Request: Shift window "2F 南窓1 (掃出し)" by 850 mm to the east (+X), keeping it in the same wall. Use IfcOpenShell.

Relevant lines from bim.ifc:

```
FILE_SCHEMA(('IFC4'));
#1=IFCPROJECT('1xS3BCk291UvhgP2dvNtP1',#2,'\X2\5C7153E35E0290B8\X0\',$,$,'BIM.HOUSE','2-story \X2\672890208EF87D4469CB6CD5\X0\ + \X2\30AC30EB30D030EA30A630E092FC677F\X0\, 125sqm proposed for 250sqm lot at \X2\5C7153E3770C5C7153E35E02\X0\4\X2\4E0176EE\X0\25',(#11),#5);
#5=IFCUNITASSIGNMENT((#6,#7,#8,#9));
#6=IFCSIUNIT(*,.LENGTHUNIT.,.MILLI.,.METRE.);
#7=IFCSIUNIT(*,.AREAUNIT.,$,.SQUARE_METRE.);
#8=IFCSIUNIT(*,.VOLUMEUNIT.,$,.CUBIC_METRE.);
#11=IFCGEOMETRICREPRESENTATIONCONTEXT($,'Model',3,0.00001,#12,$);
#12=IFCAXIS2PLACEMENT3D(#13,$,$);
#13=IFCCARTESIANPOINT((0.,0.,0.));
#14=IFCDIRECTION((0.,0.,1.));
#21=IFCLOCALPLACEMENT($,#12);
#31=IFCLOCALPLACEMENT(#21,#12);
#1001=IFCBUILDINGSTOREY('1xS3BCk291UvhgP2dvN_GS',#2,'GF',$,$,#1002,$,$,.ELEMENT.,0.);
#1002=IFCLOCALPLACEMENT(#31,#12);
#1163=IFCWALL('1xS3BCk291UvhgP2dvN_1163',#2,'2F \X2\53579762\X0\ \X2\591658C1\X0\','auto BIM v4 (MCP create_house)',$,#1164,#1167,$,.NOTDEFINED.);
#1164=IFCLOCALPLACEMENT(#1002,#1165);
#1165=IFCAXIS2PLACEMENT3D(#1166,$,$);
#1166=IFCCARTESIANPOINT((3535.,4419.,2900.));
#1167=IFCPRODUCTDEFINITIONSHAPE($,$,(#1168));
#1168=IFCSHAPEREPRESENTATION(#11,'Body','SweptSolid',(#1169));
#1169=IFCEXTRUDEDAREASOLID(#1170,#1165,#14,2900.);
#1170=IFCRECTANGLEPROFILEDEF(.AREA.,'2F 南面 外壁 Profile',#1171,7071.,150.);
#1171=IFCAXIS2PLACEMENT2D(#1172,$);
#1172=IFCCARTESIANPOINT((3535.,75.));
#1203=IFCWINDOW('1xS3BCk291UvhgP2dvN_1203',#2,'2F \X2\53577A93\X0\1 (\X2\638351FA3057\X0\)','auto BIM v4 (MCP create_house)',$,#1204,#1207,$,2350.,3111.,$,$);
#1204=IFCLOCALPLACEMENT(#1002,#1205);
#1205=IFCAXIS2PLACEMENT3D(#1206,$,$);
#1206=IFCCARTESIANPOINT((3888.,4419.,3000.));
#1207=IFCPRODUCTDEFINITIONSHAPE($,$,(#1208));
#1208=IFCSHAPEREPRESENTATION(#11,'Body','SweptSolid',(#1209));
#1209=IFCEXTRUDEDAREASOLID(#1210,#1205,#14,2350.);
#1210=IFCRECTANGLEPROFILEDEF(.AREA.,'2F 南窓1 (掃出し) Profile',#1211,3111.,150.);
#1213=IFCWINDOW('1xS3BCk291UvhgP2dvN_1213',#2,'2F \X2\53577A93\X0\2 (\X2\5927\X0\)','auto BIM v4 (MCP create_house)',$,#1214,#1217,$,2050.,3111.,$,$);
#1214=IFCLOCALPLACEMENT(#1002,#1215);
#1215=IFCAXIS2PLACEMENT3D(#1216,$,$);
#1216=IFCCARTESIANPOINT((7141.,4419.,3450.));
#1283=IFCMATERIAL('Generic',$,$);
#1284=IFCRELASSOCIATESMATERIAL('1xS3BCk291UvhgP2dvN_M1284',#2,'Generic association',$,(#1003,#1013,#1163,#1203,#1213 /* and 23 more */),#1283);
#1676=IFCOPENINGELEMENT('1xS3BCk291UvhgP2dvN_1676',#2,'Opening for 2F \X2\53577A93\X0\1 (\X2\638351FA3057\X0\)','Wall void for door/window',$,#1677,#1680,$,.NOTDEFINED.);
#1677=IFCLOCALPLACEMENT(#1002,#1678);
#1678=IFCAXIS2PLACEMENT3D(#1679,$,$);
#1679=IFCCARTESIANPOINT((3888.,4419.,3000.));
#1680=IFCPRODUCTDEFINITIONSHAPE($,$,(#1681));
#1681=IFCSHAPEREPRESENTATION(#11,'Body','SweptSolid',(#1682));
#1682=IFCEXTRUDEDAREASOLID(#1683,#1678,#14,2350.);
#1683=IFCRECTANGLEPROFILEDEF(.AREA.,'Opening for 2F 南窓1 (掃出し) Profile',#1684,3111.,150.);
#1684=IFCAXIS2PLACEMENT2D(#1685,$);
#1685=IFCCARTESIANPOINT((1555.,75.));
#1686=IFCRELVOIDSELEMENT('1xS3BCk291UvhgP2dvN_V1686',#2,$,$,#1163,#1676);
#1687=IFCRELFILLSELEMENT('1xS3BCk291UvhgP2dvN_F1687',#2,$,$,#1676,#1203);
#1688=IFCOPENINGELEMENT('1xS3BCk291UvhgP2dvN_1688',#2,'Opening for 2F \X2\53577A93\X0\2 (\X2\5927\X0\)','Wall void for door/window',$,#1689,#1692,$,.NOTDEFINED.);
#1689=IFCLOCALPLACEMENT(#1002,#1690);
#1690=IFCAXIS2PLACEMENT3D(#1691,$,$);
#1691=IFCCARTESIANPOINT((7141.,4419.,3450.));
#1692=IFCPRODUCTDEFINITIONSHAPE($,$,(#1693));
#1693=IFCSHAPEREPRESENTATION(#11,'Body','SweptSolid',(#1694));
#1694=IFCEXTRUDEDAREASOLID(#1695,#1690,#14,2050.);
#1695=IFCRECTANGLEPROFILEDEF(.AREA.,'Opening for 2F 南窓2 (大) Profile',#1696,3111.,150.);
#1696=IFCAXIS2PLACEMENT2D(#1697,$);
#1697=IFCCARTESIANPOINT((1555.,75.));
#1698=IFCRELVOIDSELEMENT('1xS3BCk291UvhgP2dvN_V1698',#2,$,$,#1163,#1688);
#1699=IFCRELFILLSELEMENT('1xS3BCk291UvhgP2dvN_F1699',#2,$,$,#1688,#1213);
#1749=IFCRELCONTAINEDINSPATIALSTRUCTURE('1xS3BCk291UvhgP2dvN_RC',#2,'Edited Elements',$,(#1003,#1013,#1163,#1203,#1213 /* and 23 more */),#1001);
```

```python
import ifcopenshell
import ifcopenshell.api.geometry
import ifcopenshell.util.placement
import ifcopenshell.util.unit

model = ifcopenshell.open("bim.ifc")
unit_scale = ifcopenshell.util.unit.calculate_unit_scale(model)

window = model.by_guid("1xS3BCk291UvhgP2dvN_1203")
opening = window.FillsVoids[0].RelatingOpeningElement
wall = opening.VoidsElements[0].RelatingBuildingElement

wall_matrix = ifcopenshell.util.placement.get_local_placement(wall.ObjectPlacement)
shift = wall_matrix[:3, 0] * 0.85 / unit_scale
before = ifcopenshell.util.placement.get_local_placement(window.ObjectPlacement)[:3, 3].copy()

# The window is not placed relative to its opening, so move both.
for product in (opening, window):
    matrix = ifcopenshell.util.placement.get_local_placement(product.ObjectPlacement)
    matrix[:3, 3] += shift
    ifcopenshell.api.geometry.edit_object_placement(model, product=product, matrix=matrix, is_si=False)

after = ifcopenshell.util.placement.get_local_placement(window.ObjectPlacement)[:3, 3]
print("window moved by", (after - before).round(3) + 0.0)

model.write("bim_v2.ifc")
```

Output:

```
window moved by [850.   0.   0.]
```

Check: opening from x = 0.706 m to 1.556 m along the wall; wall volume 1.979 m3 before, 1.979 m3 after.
